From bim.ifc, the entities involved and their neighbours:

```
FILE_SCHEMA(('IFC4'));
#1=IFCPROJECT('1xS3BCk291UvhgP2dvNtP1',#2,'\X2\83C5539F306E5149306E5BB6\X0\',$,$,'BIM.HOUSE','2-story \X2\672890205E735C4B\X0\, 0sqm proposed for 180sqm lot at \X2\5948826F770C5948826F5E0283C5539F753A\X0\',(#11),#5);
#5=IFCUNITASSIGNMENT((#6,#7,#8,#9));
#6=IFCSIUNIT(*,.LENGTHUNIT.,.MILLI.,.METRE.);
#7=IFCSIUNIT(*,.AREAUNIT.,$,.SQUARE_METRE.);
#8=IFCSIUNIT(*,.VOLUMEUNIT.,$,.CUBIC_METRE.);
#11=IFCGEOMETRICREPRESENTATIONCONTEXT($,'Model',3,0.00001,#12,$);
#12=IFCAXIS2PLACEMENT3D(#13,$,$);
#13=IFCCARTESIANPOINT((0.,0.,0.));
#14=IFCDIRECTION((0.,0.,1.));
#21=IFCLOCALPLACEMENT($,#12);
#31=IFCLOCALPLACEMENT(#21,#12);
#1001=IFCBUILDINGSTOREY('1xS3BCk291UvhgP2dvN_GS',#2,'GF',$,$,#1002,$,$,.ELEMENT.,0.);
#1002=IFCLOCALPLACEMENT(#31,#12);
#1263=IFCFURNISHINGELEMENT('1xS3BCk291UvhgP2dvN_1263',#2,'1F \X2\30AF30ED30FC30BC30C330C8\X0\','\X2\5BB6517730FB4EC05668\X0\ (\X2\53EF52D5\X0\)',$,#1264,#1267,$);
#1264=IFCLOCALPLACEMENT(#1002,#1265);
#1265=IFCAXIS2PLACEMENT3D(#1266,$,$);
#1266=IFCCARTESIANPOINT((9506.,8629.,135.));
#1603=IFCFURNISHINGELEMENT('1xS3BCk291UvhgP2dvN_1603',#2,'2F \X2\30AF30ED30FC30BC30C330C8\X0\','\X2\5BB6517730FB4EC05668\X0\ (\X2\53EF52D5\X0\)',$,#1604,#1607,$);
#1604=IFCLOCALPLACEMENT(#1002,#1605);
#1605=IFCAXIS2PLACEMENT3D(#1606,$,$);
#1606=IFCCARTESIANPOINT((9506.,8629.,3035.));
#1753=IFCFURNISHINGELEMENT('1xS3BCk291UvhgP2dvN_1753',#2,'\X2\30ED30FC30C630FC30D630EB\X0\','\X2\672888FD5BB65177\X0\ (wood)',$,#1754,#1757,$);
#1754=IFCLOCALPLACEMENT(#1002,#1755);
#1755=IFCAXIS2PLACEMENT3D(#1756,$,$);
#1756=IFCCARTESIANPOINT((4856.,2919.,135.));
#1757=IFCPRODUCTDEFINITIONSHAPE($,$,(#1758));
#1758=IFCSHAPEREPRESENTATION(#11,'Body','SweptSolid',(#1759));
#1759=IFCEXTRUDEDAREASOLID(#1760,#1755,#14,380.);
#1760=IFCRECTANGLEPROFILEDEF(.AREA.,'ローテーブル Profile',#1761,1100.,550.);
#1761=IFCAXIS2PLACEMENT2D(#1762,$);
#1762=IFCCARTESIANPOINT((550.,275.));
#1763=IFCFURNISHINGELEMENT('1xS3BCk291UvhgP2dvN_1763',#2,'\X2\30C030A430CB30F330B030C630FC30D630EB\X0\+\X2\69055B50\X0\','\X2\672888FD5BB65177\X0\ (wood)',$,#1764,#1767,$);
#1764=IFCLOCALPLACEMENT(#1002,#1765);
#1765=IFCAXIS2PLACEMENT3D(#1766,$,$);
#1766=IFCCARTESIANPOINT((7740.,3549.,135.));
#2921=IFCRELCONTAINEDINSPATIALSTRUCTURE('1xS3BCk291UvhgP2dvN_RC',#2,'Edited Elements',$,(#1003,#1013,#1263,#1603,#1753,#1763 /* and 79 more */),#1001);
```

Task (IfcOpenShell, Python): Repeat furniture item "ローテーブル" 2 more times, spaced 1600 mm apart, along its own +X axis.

```python
import ifcopenshell
import ifcopenshell.api.geometry
import ifcopenshell.api.root
import ifcopenshell.util.element
import ifcopenshell.util.placement
import ifcopenshell.util.unit

model = ifcopenshell.open("bim.ifc")
unit_scale = ifcopenshell.util.unit.calculate_unit_scale(model)


def reuse_history(source, copy):
    """copy_class also copies each property set's owner history, people and application; keep the originals."""
    for rel in copy.IsDefinedBy:
        if rel.is_a("IfcRelDefinesByProperties") and (history := rel.RelatingPropertyDefinition.OwnerHistory):
            rel.RelatingPropertyDefinition.OwnerHistory = source.OwnerHistory
            ifcopenshell.util.element.remove_deep2(model, history)


source = model.by_id(1753)
base = ifcopenshell.util.placement.get_local_placement(source.ObjectPlacement)
step = base[:3, 0] * 1.6 / unit_scale

for i in range(1, 3):
    copy = ifcopenshell.api.root.copy_class(model, product=source)
    copy.Representation = ifcopenshell.util.element.copy_deep(
        model, source.Representation, exclude=["IfcGeometricRepresentationContext", "IfcRepresentationMap"]
    )
    reuse_history(source, copy)
    matrix = base.copy()
    matrix[:3, 3] += i * step
    print("added at", matrix[:3, 3].round(3) + 0.0)
    ifcopenshell.api.geometry.edit_object_placement(model, product=copy, matrix=matrix, is_si=False)

model.write("bim_rev.ifc")
```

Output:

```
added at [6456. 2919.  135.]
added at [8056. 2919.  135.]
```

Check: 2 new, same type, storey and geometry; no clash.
